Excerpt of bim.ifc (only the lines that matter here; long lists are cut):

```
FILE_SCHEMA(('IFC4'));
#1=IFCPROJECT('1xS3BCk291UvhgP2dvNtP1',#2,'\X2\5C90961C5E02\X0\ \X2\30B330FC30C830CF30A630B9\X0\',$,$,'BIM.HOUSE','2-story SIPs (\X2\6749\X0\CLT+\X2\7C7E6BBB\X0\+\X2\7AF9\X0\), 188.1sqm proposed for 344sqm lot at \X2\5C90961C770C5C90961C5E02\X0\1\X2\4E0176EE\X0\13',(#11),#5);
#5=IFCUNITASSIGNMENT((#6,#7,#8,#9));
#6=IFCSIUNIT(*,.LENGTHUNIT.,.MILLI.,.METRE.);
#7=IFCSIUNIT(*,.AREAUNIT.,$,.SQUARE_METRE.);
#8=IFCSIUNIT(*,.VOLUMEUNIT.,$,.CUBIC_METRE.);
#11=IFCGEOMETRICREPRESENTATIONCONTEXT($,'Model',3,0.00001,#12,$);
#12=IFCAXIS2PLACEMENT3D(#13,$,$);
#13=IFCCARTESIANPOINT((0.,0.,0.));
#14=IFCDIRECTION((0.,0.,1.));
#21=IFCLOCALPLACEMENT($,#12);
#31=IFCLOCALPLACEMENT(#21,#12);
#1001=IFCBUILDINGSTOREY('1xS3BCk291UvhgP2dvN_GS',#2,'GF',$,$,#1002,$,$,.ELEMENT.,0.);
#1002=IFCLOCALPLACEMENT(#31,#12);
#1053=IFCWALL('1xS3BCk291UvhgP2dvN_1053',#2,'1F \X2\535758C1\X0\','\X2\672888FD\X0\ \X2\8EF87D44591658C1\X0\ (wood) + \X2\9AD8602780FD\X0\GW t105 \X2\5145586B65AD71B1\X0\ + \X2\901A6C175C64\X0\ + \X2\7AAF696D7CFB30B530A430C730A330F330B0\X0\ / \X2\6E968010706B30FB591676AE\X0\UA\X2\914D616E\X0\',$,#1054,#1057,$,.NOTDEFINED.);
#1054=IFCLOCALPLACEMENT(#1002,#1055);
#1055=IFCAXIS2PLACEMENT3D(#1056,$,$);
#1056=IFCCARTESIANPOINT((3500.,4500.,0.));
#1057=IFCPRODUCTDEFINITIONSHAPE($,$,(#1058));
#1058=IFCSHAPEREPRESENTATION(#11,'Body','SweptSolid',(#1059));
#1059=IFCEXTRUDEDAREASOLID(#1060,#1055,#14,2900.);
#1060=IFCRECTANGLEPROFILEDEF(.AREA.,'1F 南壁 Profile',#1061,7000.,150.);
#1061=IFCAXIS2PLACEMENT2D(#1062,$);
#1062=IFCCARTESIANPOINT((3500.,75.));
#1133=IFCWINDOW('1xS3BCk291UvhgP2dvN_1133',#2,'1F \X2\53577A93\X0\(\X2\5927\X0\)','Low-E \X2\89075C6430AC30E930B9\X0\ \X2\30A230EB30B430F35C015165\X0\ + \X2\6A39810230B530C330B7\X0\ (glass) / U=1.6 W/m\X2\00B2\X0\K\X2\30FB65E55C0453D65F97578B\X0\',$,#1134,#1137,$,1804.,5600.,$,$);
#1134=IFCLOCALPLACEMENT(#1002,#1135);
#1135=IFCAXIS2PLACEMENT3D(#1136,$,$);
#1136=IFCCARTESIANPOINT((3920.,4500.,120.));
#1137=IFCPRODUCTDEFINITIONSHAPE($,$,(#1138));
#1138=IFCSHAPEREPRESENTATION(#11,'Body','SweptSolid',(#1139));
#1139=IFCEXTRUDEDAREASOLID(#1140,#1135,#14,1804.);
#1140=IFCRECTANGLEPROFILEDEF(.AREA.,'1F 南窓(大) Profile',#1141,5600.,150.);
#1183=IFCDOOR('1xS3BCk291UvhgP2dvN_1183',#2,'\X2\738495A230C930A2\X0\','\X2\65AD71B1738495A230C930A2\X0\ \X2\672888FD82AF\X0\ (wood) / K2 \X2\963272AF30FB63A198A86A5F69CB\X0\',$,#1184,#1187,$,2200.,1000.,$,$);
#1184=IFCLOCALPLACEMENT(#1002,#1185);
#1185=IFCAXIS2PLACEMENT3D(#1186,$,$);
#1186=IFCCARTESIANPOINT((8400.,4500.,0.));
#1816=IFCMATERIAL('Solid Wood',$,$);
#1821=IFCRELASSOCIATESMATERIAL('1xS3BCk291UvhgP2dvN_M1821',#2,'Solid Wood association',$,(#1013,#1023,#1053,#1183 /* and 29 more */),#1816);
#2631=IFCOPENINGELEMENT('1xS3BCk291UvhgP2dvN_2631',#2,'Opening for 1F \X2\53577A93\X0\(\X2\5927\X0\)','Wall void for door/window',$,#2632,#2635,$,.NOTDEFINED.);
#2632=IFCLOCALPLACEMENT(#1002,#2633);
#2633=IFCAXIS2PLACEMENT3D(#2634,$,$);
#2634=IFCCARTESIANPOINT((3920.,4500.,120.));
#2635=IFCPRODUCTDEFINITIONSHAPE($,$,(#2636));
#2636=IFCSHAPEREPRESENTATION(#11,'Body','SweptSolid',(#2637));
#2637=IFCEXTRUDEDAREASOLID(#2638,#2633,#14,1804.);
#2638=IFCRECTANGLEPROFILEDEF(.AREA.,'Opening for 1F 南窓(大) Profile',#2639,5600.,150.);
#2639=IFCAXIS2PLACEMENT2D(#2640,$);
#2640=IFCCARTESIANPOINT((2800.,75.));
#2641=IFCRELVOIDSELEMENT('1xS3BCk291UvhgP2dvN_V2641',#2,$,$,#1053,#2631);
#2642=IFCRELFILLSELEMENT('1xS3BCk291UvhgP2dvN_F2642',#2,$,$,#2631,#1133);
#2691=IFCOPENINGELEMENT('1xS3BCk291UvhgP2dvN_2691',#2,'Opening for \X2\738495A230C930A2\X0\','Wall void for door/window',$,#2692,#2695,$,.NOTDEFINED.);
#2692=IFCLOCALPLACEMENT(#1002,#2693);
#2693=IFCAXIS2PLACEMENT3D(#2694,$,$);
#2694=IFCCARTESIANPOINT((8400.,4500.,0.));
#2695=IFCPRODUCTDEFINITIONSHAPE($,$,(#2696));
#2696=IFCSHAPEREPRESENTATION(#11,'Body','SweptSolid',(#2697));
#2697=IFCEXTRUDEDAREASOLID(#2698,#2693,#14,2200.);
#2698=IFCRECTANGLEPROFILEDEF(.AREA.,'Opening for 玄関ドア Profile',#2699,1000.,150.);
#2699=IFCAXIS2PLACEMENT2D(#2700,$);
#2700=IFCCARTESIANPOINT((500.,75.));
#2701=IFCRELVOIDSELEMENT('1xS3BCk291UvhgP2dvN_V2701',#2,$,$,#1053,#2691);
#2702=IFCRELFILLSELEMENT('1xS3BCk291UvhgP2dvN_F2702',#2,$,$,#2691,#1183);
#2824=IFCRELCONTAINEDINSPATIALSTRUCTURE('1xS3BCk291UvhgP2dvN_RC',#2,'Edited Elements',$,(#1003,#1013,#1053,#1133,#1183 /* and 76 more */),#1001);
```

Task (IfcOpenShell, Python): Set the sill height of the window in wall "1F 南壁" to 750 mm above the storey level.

```python
import numpy as np
import ifcopenshell
import ifcopenshell.api.geometry
import ifcopenshell.geom
import ifcopenshell.util.element
import ifcopenshell.util.placement
import ifcopenshell.util.shape
import ifcopenshell.util.unit

model = ifcopenshell.open("bim.ifc")
unit_scale = ifcopenshell.util.unit.calculate_unit_scale(model)

window = model.by_guid("1xS3BCk291UvhgP2dvN_1133")
opening = window.FillsVoids[0].RelatingOpeningElement
storey = ifcopenshell.util.element.get_container(window, ifc_class="IfcBuildingStorey")
level = ifcopenshell.util.placement.get_local_placement(storey.ObjectPlacement)[2, 3]

# The opening's origin need not be at the sill, so measure its lowest point.
shape = ifcopenshell.geom.create_shape(ifcopenshell.geom.settings(), opening)
bottom = ifcopenshell.util.shape.get_shape_bottom_elevation(shape, shape.geometry) / unit_scale
dz = level + 0.75 / unit_scale - bottom

shift = np.array([0.0, 0.0, dz])
# The window is not placed relative to its opening, so move both.
for product in (opening, window):
    matrix = ifcopenshell.util.placement.get_local_placement(product.ObjectPlacement)
    matrix[:3, 3] += shift
    ifcopenshell.api.geometry.edit_object_placement(model, product=product, matrix=matrix, is_si=False)

print(f"moved by {dz * unit_scale:+.3f} m")

model.write("bim_rev.ifc")
```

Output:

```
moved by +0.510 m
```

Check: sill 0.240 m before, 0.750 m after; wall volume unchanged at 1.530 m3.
